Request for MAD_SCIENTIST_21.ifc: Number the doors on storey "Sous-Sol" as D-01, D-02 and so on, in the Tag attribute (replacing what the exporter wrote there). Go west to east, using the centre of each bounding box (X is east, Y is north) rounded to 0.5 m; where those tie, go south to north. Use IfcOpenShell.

First a look at what the model holds.

```python
import ifcopenshell
import ifcopenshell.util.element
import ifcopenshell.util.placement

model = ifcopenshell.open("MAD_SCIENTIST_21.ifc")
print(model.schema)
storey = next(s for s in model.by_type("IfcBuildingStorey") if s.Name == "Sous-Sol")
doors = [e for e in ifcopenshell.util.element.get_decomposition(storey) if e.is_a("IfcDoor")]
for e in sorted(doors, key=lambda e: e.id()):
    origin = ifcopenshell.util.placement.get_local_placement(e.ObjectPlacement)[:3, 3]
    print(e.id(), e.Tag, e.Name, origin.round(2) + 0.0, sep=" | ")
```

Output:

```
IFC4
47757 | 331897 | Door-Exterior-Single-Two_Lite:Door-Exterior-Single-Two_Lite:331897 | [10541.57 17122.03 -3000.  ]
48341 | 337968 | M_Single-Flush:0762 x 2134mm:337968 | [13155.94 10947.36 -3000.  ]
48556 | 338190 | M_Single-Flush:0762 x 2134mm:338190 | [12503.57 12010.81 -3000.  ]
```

```python
import ifcopenshell
import ifcopenshell.geom
import ifcopenshell.util.element
import ifcopenshell.util.shape

model = ifcopenshell.open("MAD_SCIENTIST_21.ifc")
settings = ifcopenshell.geom.settings()
settings.set("use-world-coords", True)


def centre(element):
    shape = ifcopenshell.geom.create_shape(settings, element)
    return ifcopenshell.util.shape.get_bbox_centroid(shape.geometry)


storey = next(s for s in model.by_type("IfcBuildingStorey") if s.Name == "Sous-Sol")
doors = [e for e in ifcopenshell.util.element.get_decomposition(storey) if e.is_a("IfcDoor")]

# Insertion points can sit at a corner or the storey origin, so sort by the geometry (in metres).
centres = {e: centre(e) for e in doors}
doors.sort(key=lambda e: (round(centres[e][0] / 0.5), centres[e][1]))

for i, e in enumerate(doors, start=1):
    number = f"D-{i:02d}"
    e.Tag = number
    print(e.id(), number)

model.write("MAD_SCIENTIST_21_v2.ifc")
```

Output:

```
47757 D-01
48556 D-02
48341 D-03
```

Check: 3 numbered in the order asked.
